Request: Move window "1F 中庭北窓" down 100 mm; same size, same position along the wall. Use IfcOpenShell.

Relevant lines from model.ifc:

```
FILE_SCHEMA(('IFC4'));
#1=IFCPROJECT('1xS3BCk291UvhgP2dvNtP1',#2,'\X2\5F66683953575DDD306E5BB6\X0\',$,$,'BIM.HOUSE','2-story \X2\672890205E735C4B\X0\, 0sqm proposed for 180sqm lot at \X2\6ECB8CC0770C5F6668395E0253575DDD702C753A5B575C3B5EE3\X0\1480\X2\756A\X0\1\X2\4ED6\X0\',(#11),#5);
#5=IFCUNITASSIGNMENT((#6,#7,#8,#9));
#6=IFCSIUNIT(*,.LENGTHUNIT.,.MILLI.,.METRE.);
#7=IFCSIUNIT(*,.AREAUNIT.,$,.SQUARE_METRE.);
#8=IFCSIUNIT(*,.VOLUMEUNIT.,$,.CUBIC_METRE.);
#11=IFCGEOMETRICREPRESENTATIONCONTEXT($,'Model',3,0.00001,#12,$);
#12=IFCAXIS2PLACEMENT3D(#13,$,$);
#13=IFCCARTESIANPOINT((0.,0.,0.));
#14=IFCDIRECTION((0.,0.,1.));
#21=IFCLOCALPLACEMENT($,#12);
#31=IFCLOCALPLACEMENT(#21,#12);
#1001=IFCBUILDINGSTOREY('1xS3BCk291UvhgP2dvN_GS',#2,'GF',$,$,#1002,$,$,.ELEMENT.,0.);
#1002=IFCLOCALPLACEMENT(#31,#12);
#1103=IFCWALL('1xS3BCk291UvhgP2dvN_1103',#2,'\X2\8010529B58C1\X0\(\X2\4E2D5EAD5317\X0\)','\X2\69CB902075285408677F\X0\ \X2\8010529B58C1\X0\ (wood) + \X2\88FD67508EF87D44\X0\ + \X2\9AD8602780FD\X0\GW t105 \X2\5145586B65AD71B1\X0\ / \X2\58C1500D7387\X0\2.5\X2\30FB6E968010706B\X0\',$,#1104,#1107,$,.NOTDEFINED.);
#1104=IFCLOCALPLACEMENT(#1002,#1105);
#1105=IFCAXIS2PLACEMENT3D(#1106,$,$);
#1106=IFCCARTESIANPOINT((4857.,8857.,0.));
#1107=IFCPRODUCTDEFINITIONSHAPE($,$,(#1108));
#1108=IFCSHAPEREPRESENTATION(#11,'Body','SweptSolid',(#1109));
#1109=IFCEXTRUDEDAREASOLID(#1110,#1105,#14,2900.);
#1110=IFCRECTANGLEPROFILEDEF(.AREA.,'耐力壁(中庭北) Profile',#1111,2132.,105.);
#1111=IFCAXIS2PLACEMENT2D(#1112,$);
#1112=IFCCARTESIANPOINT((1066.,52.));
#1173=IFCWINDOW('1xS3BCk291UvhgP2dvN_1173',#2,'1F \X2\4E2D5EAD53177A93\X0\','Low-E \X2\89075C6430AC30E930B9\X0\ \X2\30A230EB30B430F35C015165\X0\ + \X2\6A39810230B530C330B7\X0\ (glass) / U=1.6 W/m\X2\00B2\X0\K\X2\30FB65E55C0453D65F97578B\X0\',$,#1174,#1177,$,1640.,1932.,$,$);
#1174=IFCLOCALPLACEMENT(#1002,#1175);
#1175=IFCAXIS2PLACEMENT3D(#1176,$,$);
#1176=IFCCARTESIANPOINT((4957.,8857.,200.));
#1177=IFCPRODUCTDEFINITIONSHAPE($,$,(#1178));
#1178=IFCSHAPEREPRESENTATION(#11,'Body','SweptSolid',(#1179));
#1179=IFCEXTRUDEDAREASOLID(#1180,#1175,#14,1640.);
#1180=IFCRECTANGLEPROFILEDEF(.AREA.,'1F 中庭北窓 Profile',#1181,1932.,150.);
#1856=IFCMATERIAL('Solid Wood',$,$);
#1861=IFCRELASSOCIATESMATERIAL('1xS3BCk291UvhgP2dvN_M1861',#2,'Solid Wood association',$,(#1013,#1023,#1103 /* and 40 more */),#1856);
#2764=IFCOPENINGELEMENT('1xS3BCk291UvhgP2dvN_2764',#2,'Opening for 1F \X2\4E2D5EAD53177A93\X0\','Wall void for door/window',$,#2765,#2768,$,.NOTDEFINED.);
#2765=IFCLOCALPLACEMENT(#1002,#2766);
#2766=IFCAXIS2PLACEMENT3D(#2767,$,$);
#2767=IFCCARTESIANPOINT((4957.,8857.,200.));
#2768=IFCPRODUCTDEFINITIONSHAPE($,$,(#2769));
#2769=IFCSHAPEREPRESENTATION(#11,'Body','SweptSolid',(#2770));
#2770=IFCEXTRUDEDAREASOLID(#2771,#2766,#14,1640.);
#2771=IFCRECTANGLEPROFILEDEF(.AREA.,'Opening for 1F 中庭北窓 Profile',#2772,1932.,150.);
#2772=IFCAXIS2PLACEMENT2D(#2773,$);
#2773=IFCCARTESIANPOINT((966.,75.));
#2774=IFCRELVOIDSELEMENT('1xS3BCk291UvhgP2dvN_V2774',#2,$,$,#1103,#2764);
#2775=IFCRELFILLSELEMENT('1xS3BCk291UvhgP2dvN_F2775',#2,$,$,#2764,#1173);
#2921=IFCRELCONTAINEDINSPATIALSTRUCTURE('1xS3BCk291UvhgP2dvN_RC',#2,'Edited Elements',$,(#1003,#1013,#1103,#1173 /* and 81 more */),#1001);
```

```python
import numpy as np
import ifcopenshell
import ifcopenshell.api.geometry
import ifcopenshell.util.placement
import ifcopenshell.util.unit

model = ifcopenshell.open("model.ifc")
unit_scale = ifcopenshell.util.unit.calculate_unit_scale(model)

window = model.by_guid("1xS3BCk291UvhgP2dvN_1173")
opening = window.FillsVoids[0].RelatingOpeningElement
dz = -0.1 / unit_scale

shift = np.array([0.0, 0.0, dz])
# The window is not placed relative to its opening, so move both.
for product in (opening, window):
    matrix = ifcopenshell.util.placement.get_local_placement(product.ObjectPlacement)
    matrix[:3, 3] += shift
    ifcopenshell.api.geometry.edit_object_placement(model, product=product, matrix=matrix, is_si=False)

print(f"moved by {dz * unit_scale:+.3f} m")

model.write("model_edited.ifc")
```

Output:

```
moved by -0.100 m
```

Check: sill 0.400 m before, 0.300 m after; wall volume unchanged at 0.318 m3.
